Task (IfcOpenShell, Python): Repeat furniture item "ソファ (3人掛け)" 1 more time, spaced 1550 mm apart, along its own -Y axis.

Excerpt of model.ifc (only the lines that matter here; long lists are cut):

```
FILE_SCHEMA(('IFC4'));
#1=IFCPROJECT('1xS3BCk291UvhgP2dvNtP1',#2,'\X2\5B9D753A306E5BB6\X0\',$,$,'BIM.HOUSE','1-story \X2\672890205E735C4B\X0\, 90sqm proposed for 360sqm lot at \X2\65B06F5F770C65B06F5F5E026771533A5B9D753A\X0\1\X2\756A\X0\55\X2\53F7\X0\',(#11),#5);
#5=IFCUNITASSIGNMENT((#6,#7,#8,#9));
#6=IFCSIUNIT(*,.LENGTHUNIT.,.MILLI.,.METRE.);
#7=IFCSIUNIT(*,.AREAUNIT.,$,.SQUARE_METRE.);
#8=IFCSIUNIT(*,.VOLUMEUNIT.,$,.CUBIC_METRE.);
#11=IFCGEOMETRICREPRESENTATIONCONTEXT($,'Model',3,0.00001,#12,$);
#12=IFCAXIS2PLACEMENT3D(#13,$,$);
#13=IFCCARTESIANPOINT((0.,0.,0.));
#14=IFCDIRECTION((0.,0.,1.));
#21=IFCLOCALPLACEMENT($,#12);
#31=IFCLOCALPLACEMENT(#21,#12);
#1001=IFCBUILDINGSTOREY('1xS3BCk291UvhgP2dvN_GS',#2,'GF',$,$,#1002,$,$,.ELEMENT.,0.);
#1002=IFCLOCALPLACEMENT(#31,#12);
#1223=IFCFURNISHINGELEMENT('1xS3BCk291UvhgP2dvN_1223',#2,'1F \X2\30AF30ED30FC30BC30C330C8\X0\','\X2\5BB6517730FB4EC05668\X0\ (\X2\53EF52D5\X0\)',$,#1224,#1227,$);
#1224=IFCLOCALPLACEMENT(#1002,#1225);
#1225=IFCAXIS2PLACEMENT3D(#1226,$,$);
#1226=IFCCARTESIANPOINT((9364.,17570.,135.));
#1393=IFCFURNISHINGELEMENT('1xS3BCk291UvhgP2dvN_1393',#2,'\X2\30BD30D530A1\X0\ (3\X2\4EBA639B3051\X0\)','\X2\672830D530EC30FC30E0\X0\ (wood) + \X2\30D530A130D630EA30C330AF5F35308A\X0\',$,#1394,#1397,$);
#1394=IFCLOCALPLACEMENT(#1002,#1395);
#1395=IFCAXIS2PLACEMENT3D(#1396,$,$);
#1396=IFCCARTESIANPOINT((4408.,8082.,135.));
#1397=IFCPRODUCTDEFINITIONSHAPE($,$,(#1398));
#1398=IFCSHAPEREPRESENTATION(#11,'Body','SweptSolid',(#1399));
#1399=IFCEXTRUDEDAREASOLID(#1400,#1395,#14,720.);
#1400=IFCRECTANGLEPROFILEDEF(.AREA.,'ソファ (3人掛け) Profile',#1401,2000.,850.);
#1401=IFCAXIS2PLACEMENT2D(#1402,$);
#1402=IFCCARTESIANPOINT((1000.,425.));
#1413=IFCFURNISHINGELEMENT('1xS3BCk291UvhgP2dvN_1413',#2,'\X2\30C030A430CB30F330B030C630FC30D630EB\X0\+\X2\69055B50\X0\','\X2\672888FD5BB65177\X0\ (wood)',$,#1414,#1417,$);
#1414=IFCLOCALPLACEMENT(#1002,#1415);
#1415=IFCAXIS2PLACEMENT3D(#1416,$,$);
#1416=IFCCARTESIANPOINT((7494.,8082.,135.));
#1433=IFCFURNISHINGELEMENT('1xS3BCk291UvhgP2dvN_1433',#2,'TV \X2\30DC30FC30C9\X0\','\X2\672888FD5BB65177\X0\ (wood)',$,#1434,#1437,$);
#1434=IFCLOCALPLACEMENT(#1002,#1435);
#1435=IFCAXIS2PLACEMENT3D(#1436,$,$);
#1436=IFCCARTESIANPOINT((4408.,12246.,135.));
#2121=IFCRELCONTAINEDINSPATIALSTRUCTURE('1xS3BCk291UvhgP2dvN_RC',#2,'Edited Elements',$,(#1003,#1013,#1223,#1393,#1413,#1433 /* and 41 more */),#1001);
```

```python
import ifcopenshell
import ifcopenshell.api.geometry
import ifcopenshell.api.root
import ifcopenshell.util.element
import ifcopenshell.util.placement
import ifcopenshell.util.unit

model = ifcopenshell.open("model.ifc")
unit_scale = ifcopenshell.util.unit.calculate_unit_scale(model)


def reuse_history(source, copy):
    """copy_class also copies each property set's owner history, people and application; keep the originals."""
    for rel in copy.IsDefinedBy:
        if rel.is_a("IfcRelDefinesByProperties") and (history := rel.RelatingPropertyDefinition.OwnerHistory):
            rel.RelatingPropertyDefinition.OwnerHistory = source.OwnerHistory
            ifcopenshell.util.element.remove_deep2(model, history)


source = model.by_id(1393)
base = ifcopenshell.util.placement.get_local_placement(source.ObjectPlacement)
step = -base[:3, 1] * 1.55 / unit_scale

for i in range(1, 2):
    copy = ifcopenshell.api.root.copy_class(model, product=source)
    copy.Representation = ifcopenshell.util.element.copy_deep(
        model, source.Representation, exclude=["IfcGeometricRepresentationContext", "IfcRepresentationMap"]
    )
    reuse_history(source, copy)
    matrix = base.copy()
    matrix[:3, 3] += i * step
    print("added at", matrix[:3, 3].round(3) + 0.0)
    ifcopenshell.api.geometry.edit_object_placement(model, product=copy, matrix=matrix, is_si=False)

model.write("model_updated.ifc")
```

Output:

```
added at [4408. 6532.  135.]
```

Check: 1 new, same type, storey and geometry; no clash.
